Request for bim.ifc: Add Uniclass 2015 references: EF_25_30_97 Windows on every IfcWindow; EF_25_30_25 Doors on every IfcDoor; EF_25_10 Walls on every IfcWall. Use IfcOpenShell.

First a look at what the model holds.

```python
import ifcopenshell

model = ifcopenshell.open("bim.ifc")
print(model.schema)
print("classifications:", [c.Name for c in model.by_type("IfcClassification")])
for ifc_class in ("IfcDoor", "IfcRoof", "IfcStair", "IfcWall", "IfcWindow"):
    print(ifc_class, len(model.by_type(ifc_class)))
```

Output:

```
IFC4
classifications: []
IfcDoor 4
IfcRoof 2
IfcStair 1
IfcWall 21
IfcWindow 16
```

```python
import ifcopenshell
import ifcopenshell.api.classification

model = ifcopenshell.open("bim.ifc")

system = ifcopenshell.api.classification.add_classification(model, classification="Uniclass 2015")

codes = {
    "IfcWindow": ("EF_25_30_97", "Windows"),
    "IfcDoor": ("EF_25_30_25", "Doors"),
    "IfcWall": ("EF_25_10", "Walls"),
}
for ifc_class, (code, name) in codes.items():
    products = model.by_type(ifc_class)
    ifcopenshell.api.classification.add_reference(
        model, products=products, classification=system, identification=code, name=name
    )
    print(code, len(products))

model.write("bim_rev.ifc")
```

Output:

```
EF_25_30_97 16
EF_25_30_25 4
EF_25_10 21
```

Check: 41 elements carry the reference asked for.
